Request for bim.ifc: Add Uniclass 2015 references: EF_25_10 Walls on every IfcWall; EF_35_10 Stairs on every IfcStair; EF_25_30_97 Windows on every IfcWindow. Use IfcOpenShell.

First a look at what the model holds.

```python
import ifcopenshell

model = ifcopenshell.open("bim.ifc")
print(model.schema)
print("classifications:", [c.Name for c in model.by_type("IfcClassification")])
for ifc_class in ("IfcDoor", "IfcRoof", "IfcStair", "IfcWall", "IfcWindow"):
    print(ifc_class, len(model.by_type(ifc_class)))
```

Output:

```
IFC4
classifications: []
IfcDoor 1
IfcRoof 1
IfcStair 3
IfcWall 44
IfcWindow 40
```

```python
import ifcopenshell
import ifcopenshell.api.classification

model = ifcopenshell.open("bim.ifc")

system = ifcopenshell.api.classification.add_classification(model, classification="Uniclass 2015")

codes = {
    "IfcWall": ("EF_25_10", "Walls"),
    "IfcStair": ("EF_35_10", "Stairs"),
    "IfcWindow": ("EF_25_30_97", "Windows"),
}
for ifc_class, (code, name) in codes.items():
    products = model.by_type(ifc_class)
    ifcopenshell.api.classification.add_reference(
        model, products=products, classification=system, identification=code, name=name
    )
    print(code, len(products))

model.write("bim_rev.ifc")
```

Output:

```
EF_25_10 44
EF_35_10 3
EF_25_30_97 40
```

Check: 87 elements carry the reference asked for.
